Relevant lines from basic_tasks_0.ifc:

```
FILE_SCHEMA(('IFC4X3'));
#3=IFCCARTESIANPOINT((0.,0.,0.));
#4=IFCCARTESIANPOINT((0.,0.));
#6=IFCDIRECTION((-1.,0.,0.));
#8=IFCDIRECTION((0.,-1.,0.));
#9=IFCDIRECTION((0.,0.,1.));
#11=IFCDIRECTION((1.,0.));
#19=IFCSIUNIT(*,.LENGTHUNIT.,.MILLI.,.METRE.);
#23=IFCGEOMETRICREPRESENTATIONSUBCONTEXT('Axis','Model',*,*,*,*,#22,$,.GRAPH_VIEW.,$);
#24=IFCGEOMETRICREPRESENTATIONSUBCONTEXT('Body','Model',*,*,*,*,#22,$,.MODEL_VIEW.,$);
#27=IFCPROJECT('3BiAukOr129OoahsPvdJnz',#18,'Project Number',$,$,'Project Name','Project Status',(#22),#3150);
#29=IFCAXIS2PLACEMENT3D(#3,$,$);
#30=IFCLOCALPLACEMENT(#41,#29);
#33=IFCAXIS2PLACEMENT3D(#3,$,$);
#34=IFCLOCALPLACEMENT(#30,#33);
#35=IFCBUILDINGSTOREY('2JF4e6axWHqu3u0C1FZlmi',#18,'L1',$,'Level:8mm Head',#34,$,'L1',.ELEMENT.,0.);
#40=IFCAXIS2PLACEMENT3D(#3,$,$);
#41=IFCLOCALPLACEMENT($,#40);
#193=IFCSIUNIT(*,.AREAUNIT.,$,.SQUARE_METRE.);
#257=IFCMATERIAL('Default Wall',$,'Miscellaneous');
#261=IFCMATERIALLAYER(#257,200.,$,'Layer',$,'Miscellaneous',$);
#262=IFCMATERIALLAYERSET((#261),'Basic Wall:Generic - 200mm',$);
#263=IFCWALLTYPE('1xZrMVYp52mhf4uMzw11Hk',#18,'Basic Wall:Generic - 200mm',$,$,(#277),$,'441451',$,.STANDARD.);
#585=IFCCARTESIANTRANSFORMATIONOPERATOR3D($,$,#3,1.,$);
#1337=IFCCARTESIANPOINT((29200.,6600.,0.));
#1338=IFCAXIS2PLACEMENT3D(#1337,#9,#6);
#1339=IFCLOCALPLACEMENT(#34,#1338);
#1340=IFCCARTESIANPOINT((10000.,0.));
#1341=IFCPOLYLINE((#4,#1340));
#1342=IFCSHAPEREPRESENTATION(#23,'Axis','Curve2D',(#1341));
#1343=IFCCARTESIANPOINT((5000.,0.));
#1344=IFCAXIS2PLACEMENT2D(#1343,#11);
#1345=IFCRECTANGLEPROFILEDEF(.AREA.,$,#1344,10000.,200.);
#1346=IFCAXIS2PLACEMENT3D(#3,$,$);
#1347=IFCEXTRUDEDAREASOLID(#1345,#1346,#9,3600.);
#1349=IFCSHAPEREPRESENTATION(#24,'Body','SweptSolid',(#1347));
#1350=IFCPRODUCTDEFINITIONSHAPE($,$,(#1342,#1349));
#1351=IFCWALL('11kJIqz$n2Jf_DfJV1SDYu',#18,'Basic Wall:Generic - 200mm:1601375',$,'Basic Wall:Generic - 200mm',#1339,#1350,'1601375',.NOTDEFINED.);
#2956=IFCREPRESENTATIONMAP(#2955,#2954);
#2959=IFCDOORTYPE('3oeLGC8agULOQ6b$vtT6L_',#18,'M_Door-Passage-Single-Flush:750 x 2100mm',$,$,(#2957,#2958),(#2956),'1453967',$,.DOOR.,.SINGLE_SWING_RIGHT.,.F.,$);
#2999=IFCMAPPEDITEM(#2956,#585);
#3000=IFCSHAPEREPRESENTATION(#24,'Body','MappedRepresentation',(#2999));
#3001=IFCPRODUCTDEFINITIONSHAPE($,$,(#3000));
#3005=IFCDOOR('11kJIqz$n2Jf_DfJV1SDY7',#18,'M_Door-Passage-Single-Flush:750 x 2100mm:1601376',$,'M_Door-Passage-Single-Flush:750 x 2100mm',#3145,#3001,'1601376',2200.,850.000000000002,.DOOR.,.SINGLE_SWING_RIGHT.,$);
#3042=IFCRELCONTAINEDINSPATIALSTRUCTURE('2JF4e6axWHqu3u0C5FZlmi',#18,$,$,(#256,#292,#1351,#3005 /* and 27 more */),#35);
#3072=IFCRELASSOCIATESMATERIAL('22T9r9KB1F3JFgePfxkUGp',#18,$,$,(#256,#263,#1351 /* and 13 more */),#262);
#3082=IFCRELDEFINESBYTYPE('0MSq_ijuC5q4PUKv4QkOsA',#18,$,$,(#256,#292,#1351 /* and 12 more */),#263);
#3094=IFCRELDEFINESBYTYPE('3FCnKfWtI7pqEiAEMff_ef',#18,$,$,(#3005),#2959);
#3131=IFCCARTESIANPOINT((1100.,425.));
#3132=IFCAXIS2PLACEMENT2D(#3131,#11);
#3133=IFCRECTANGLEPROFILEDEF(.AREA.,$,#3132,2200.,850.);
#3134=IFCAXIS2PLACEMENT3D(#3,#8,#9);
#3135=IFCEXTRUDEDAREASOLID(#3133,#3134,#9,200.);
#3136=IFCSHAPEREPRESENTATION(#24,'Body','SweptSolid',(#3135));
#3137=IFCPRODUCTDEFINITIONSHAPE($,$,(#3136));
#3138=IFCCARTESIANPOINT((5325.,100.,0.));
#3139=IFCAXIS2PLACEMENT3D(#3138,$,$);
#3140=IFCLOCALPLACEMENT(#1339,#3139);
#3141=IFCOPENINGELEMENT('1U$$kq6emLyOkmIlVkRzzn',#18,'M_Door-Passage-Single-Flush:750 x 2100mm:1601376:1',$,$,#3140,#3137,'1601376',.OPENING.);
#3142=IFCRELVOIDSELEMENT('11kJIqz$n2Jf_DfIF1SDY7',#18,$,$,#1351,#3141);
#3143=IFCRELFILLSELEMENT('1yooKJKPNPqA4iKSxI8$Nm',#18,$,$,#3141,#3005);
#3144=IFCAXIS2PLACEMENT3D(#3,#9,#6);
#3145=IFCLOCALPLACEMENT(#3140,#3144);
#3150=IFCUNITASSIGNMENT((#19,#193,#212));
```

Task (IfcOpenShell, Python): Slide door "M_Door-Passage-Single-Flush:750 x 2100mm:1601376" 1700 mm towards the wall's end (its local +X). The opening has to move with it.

```python
import ifcopenshell
import ifcopenshell.api.geometry
import ifcopenshell.util.placement
import ifcopenshell.util.unit

model = ifcopenshell.open("basic_tasks_0.ifc")
unit_scale = ifcopenshell.util.unit.calculate_unit_scale(model)

door = model.by_id(3005)
opening = door.FillsVoids[0].RelatingOpeningElement
wall = opening.VoidsElements[0].RelatingBuildingElement

wall_matrix = ifcopenshell.util.placement.get_local_placement(wall.ObjectPlacement)
shift = wall_matrix[:3, 0] * 1.7 / unit_scale
before = ifcopenshell.util.placement.get_local_placement(door.ObjectPlacement)[:3, 3].copy()

# The door is placed relative to its opening, so it follows when the opening moves.
matrix = ifcopenshell.util.placement.get_local_placement(opening.ObjectPlacement)
matrix[:3, 3] += shift
ifcopenshell.api.geometry.edit_object_placement(
    model, product=opening, matrix=matrix, is_si=False, should_transform_children=True
)

after = ifcopenshell.util.placement.get_local_placement(door.ObjectPlacement)[:3, 3]
print("door moved by", (after - before).round(3) + 0.0)

model.write("basic_tasks_0_rev.ifc")
```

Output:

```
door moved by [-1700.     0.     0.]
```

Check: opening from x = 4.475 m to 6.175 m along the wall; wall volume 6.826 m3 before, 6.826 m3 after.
